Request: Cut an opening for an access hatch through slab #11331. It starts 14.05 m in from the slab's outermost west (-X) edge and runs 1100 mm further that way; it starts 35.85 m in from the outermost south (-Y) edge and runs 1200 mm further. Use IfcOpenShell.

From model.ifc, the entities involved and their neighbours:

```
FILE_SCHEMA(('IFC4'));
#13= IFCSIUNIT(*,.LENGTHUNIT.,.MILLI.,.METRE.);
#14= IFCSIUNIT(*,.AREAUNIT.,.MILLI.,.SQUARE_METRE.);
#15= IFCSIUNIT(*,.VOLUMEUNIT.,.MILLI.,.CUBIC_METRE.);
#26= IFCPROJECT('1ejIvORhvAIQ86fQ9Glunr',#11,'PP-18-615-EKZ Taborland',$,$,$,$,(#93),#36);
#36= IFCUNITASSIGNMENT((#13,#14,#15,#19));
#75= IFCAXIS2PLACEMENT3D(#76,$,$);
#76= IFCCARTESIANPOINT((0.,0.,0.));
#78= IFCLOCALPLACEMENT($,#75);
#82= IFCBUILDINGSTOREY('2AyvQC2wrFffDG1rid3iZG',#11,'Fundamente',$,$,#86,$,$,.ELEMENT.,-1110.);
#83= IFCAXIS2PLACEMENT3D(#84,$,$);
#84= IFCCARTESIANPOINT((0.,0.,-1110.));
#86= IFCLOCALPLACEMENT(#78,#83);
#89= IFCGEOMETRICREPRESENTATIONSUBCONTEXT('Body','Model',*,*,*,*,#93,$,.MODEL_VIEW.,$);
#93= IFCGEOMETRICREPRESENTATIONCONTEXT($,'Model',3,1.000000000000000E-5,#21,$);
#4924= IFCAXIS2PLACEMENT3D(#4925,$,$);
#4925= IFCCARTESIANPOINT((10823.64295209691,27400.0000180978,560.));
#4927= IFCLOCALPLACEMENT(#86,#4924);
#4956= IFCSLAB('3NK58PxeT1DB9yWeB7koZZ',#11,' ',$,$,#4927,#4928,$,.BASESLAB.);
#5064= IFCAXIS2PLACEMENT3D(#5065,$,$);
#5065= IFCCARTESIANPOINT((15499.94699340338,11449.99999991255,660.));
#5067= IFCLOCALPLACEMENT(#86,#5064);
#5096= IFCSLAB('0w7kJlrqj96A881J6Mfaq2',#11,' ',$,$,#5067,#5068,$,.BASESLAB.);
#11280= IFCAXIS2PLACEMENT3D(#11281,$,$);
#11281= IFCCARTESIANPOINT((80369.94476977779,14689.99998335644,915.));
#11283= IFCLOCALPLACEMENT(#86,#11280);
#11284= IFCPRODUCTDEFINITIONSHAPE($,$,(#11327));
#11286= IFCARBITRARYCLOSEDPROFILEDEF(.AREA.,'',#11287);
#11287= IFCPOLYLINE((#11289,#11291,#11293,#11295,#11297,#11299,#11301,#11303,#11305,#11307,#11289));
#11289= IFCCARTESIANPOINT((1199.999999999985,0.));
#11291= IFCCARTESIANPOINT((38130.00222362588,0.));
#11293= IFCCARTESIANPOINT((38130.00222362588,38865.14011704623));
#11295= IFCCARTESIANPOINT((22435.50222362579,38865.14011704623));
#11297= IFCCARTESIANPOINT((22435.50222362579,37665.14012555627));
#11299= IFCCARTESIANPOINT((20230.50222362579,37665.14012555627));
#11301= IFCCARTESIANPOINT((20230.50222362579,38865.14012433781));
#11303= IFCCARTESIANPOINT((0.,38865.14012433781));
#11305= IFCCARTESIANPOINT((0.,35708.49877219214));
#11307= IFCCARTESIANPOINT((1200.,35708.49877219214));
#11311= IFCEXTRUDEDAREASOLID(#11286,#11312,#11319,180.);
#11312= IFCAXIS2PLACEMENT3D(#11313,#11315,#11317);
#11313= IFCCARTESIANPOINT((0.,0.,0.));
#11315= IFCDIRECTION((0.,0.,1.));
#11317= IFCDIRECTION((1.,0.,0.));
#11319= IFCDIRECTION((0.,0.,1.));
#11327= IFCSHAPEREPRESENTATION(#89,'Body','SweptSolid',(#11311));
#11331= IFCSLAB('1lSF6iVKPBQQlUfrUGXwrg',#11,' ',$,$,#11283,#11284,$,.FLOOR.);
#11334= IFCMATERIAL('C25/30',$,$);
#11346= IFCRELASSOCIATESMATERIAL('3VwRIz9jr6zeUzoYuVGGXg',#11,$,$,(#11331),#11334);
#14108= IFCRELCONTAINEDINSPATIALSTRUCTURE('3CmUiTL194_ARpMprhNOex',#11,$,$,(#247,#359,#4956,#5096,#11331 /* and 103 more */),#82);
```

```python
import numpy as np
import ifcopenshell
import ifcopenshell.api.feature
import ifcopenshell.api.geometry
import ifcopenshell.api.root
import ifcopenshell.geom
import ifcopenshell.util.placement
import ifcopenshell.util.representation
import ifcopenshell.util.shape
import ifcopenshell.util.unit

model = ifcopenshell.open("model.ifc")
unit_scale = ifcopenshell.util.unit.calculate_unit_scale(model)
settings = ifcopenshell.geom.settings()


def volume(element):
    """Net volume in cubic metres, openings subtracted."""
    shape = ifcopenshell.geom.create_shape(settings, element)
    return ifcopenshell.util.shape.get_volume(shape.geometry)


slab = model.by_guid("1lSF6iVKPBQQlUfrUGXwrg")
before = volume(slab)

# Extent in the slab's own axes, in metres. The edges named are its -X and -Y sides.
slab_shape = ifcopenshell.geom.create_shape(settings, slab)
vertices = ifcopenshell.util.shape.get_vertices(slab_shape.geometry)
x_min, y_min, bottom = vertices.min(axis=0)
top = vertices[:, 2].max()

opening = ifcopenshell.api.root.create_entity(model, ifc_class="IfcOpeningElement", name="Access hatch opening", predefined_type="OPENING")
context = ifcopenshell.util.representation.get_context(model, "Model", "Body", "MODEL_VIEW")
width, depth = 1.1, 1.2
outline = [(0.0, 0.0), (width, 0.0), (width, depth), (0.0, depth), (0.0, 0.0)]
# Overshoot both faces by 50 mm so the cut is clean.
shape = ifcopenshell.api.geometry.add_slab_representation(
    model, context=context, depth=top - bottom + 0.1, polyline=outline
)
ifcopenshell.api.geometry.assign_representation(model, product=opening, representation=shape)

matrix = ifcopenshell.util.placement.get_local_placement(slab.ObjectPlacement)
matrix[:, 3] = matrix @ np.append(np.array([x_min + 14.05, y_min + 35.85, bottom - 0.05]) / unit_scale, 1.0)
ifcopenshell.api.geometry.edit_object_placement(model, product=opening, matrix=matrix, is_si=False)
ifcopenshell.api.feature.add_feature(model, feature=opening, element=slab)

after = volume(slab)

print(f"slab volume {before:.3f} -> {after:.3f} m3")

model.write("model_rev.ifc")
```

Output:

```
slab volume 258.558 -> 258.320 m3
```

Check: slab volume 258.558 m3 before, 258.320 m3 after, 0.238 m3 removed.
